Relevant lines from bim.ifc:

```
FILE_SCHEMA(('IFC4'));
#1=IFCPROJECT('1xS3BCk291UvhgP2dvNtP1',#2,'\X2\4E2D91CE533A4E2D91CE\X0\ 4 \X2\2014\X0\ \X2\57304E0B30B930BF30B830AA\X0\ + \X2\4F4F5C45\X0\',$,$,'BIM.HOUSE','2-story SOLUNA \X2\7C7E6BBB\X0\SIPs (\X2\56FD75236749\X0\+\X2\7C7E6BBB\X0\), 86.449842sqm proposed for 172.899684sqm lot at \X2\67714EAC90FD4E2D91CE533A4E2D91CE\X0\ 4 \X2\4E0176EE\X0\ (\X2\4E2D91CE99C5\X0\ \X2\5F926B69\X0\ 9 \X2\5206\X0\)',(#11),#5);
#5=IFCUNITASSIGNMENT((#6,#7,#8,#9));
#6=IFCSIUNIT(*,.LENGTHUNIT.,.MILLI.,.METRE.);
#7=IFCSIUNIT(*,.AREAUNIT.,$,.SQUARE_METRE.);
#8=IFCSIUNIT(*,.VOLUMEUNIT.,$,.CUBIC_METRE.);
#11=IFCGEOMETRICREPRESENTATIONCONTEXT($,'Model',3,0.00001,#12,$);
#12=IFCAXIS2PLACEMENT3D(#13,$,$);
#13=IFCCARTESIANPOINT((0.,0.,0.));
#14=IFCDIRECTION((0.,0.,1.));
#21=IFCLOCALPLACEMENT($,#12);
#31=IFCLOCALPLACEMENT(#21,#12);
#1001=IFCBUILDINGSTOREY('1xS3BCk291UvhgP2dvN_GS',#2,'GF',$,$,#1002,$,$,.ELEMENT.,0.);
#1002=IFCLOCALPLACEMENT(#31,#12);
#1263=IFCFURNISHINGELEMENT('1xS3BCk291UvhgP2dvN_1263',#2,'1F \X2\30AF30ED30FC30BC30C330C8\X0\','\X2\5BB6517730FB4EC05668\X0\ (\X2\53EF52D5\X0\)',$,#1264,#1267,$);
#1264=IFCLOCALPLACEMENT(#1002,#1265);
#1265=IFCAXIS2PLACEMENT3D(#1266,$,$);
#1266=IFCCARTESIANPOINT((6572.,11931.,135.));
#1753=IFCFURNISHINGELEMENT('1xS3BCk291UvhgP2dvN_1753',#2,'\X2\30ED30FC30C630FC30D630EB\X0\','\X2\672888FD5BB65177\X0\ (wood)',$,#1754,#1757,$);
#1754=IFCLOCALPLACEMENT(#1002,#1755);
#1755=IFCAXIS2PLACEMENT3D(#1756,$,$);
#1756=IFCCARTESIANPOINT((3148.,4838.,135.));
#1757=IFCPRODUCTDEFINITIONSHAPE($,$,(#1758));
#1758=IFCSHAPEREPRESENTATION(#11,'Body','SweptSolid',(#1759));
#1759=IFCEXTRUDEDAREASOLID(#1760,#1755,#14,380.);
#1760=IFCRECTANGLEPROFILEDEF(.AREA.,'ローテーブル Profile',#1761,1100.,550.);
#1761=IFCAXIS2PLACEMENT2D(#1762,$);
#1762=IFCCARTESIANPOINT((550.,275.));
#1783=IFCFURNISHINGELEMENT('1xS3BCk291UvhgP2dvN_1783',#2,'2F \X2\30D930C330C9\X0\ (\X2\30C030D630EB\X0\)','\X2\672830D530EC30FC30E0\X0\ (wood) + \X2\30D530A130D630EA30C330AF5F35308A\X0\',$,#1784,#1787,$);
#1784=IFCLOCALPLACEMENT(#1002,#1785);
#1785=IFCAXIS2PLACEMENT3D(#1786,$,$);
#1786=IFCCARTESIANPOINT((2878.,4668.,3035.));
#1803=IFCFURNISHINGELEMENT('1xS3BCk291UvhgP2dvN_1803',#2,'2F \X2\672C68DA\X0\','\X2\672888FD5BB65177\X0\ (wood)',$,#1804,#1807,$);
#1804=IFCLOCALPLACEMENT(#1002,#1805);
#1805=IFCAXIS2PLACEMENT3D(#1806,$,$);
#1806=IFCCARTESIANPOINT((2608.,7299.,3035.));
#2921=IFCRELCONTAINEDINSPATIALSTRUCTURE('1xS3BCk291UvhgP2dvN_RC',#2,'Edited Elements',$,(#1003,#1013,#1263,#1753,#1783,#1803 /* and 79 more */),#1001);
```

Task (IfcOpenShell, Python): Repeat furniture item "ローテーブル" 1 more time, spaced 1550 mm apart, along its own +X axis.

```python
import ifcopenshell
import ifcopenshell.api.geometry
import ifcopenshell.api.root
import ifcopenshell.util.element
import ifcopenshell.util.placement
import ifcopenshell.util.unit

model = ifcopenshell.open("bim.ifc")
unit_scale = ifcopenshell.util.unit.calculate_unit_scale(model)


def reuse_history(source, copy):
    """copy_class also copies each property set's owner history, people and application; keep the originals."""
    for rel in copy.IsDefinedBy:
        if rel.is_a("IfcRelDefinesByProperties") and (history := rel.RelatingPropertyDefinition.OwnerHistory):
            rel.RelatingPropertyDefinition.OwnerHistory = source.OwnerHistory
            ifcopenshell.util.element.remove_deep2(model, history)


source = model.by_guid("1xS3BCk291UvhgP2dvN_1753")
base = ifcopenshell.util.placement.get_local_placement(source.ObjectPlacement)
step = base[:3, 0] * 1.55 / unit_scale

for i in range(1, 2):
    copy = ifcopenshell.api.root.copy_class(model, product=source)
    copy.Representation = ifcopenshell.util.element.copy_deep(
        model, source.Representation, exclude=["IfcGeometricRepresentationContext", "IfcRepresentationMap"]
    )
    reuse_history(source, copy)
    matrix = base.copy()
    matrix[:3, 3] += i * step
    print("added at", matrix[:3, 3].round(3) + 0.0)
    ifcopenshell.api.geometry.edit_object_placement(model, product=copy, matrix=matrix, is_si=False)

model.write("bim_updated.ifc")
```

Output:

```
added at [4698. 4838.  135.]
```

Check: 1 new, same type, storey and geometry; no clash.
